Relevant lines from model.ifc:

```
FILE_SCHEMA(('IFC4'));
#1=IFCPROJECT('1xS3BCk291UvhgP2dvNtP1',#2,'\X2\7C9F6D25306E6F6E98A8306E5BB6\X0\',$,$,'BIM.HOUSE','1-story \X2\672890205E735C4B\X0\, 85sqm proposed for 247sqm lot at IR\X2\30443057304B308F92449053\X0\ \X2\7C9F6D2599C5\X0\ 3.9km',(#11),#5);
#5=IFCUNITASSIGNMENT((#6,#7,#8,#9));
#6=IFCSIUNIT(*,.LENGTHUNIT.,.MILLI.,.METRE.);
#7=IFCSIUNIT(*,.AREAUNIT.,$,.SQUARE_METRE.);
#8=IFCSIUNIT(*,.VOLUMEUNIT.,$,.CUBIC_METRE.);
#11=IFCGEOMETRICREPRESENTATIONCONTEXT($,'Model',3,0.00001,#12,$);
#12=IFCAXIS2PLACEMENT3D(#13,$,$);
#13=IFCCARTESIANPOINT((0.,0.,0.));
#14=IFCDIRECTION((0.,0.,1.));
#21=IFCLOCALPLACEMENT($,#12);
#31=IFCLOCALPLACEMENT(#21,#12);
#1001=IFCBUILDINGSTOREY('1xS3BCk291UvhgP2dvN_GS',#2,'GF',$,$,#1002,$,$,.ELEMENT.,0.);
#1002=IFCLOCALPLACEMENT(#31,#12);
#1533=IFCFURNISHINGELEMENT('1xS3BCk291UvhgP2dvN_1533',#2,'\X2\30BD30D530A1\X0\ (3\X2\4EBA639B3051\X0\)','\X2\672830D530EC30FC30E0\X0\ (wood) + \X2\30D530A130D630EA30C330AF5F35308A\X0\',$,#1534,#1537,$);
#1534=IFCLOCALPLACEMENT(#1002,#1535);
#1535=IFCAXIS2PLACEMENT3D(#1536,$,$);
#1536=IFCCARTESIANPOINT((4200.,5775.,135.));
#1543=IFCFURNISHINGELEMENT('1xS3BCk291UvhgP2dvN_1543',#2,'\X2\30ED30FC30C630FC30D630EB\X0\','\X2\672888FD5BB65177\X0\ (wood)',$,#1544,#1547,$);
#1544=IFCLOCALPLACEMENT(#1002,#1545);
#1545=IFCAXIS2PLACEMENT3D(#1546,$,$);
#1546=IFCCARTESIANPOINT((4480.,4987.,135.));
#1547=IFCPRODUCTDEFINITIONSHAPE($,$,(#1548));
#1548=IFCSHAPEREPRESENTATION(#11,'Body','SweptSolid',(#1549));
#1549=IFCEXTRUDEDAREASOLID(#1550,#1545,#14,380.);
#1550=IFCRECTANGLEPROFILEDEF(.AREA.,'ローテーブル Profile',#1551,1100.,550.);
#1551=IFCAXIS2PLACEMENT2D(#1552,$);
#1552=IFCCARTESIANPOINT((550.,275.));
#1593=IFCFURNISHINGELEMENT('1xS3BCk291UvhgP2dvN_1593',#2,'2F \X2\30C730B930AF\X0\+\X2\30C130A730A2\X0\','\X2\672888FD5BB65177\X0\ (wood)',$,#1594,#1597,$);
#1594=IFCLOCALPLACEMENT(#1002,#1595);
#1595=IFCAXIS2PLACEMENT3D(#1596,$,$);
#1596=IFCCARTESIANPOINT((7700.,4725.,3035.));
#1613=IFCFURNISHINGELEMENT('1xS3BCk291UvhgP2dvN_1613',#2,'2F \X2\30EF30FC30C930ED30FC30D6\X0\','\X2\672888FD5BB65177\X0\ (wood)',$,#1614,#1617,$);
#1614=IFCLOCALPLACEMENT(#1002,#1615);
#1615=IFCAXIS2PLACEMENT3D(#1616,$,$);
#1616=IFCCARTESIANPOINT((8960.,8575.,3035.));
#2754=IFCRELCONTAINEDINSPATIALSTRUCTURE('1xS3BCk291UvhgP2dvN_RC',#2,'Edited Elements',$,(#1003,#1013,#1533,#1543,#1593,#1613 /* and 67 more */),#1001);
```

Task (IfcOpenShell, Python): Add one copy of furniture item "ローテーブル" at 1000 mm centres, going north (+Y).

```python
import numpy as np
import ifcopenshell
import ifcopenshell.api.geometry
import ifcopenshell.api.root
import ifcopenshell.util.element
import ifcopenshell.util.placement
import ifcopenshell.util.unit

model = ifcopenshell.open("model.ifc")
unit_scale = ifcopenshell.util.unit.calculate_unit_scale(model)


def reuse_history(source, copy):
    """copy_class also copies each property set's owner history, people and application; keep the originals."""
    for rel in copy.IsDefinedBy:
        if rel.is_a("IfcRelDefinesByProperties") and (history := rel.RelatingPropertyDefinition.OwnerHistory):
            rel.RelatingPropertyDefinition.OwnerHistory = source.OwnerHistory
            ifcopenshell.util.element.remove_deep2(model, history)


source = model.by_guid("1xS3BCk291UvhgP2dvN_1543")
base = ifcopenshell.util.placement.get_local_placement(source.ObjectPlacement)
step = np.array([0.0, 1.0, 0.0]) * 1 / unit_scale

for i in range(1, 2):
    copy = ifcopenshell.api.root.copy_class(model, product=source)
    copy.Representation = ifcopenshell.util.element.copy_deep(
        model, source.Representation, exclude=["IfcGeometricRepresentationContext", "IfcRepresentationMap"]
    )
    reuse_history(source, copy)
    matrix = base.copy()
    matrix[:3, 3] += i * step
    print("added at", matrix[:3, 3].round(3) + 0.0)
    ifcopenshell.api.geometry.edit_object_placement(model, product=copy, matrix=matrix, is_si=False)

model.write("model_v2.ifc")
```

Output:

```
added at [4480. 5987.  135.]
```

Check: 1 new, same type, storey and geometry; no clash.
